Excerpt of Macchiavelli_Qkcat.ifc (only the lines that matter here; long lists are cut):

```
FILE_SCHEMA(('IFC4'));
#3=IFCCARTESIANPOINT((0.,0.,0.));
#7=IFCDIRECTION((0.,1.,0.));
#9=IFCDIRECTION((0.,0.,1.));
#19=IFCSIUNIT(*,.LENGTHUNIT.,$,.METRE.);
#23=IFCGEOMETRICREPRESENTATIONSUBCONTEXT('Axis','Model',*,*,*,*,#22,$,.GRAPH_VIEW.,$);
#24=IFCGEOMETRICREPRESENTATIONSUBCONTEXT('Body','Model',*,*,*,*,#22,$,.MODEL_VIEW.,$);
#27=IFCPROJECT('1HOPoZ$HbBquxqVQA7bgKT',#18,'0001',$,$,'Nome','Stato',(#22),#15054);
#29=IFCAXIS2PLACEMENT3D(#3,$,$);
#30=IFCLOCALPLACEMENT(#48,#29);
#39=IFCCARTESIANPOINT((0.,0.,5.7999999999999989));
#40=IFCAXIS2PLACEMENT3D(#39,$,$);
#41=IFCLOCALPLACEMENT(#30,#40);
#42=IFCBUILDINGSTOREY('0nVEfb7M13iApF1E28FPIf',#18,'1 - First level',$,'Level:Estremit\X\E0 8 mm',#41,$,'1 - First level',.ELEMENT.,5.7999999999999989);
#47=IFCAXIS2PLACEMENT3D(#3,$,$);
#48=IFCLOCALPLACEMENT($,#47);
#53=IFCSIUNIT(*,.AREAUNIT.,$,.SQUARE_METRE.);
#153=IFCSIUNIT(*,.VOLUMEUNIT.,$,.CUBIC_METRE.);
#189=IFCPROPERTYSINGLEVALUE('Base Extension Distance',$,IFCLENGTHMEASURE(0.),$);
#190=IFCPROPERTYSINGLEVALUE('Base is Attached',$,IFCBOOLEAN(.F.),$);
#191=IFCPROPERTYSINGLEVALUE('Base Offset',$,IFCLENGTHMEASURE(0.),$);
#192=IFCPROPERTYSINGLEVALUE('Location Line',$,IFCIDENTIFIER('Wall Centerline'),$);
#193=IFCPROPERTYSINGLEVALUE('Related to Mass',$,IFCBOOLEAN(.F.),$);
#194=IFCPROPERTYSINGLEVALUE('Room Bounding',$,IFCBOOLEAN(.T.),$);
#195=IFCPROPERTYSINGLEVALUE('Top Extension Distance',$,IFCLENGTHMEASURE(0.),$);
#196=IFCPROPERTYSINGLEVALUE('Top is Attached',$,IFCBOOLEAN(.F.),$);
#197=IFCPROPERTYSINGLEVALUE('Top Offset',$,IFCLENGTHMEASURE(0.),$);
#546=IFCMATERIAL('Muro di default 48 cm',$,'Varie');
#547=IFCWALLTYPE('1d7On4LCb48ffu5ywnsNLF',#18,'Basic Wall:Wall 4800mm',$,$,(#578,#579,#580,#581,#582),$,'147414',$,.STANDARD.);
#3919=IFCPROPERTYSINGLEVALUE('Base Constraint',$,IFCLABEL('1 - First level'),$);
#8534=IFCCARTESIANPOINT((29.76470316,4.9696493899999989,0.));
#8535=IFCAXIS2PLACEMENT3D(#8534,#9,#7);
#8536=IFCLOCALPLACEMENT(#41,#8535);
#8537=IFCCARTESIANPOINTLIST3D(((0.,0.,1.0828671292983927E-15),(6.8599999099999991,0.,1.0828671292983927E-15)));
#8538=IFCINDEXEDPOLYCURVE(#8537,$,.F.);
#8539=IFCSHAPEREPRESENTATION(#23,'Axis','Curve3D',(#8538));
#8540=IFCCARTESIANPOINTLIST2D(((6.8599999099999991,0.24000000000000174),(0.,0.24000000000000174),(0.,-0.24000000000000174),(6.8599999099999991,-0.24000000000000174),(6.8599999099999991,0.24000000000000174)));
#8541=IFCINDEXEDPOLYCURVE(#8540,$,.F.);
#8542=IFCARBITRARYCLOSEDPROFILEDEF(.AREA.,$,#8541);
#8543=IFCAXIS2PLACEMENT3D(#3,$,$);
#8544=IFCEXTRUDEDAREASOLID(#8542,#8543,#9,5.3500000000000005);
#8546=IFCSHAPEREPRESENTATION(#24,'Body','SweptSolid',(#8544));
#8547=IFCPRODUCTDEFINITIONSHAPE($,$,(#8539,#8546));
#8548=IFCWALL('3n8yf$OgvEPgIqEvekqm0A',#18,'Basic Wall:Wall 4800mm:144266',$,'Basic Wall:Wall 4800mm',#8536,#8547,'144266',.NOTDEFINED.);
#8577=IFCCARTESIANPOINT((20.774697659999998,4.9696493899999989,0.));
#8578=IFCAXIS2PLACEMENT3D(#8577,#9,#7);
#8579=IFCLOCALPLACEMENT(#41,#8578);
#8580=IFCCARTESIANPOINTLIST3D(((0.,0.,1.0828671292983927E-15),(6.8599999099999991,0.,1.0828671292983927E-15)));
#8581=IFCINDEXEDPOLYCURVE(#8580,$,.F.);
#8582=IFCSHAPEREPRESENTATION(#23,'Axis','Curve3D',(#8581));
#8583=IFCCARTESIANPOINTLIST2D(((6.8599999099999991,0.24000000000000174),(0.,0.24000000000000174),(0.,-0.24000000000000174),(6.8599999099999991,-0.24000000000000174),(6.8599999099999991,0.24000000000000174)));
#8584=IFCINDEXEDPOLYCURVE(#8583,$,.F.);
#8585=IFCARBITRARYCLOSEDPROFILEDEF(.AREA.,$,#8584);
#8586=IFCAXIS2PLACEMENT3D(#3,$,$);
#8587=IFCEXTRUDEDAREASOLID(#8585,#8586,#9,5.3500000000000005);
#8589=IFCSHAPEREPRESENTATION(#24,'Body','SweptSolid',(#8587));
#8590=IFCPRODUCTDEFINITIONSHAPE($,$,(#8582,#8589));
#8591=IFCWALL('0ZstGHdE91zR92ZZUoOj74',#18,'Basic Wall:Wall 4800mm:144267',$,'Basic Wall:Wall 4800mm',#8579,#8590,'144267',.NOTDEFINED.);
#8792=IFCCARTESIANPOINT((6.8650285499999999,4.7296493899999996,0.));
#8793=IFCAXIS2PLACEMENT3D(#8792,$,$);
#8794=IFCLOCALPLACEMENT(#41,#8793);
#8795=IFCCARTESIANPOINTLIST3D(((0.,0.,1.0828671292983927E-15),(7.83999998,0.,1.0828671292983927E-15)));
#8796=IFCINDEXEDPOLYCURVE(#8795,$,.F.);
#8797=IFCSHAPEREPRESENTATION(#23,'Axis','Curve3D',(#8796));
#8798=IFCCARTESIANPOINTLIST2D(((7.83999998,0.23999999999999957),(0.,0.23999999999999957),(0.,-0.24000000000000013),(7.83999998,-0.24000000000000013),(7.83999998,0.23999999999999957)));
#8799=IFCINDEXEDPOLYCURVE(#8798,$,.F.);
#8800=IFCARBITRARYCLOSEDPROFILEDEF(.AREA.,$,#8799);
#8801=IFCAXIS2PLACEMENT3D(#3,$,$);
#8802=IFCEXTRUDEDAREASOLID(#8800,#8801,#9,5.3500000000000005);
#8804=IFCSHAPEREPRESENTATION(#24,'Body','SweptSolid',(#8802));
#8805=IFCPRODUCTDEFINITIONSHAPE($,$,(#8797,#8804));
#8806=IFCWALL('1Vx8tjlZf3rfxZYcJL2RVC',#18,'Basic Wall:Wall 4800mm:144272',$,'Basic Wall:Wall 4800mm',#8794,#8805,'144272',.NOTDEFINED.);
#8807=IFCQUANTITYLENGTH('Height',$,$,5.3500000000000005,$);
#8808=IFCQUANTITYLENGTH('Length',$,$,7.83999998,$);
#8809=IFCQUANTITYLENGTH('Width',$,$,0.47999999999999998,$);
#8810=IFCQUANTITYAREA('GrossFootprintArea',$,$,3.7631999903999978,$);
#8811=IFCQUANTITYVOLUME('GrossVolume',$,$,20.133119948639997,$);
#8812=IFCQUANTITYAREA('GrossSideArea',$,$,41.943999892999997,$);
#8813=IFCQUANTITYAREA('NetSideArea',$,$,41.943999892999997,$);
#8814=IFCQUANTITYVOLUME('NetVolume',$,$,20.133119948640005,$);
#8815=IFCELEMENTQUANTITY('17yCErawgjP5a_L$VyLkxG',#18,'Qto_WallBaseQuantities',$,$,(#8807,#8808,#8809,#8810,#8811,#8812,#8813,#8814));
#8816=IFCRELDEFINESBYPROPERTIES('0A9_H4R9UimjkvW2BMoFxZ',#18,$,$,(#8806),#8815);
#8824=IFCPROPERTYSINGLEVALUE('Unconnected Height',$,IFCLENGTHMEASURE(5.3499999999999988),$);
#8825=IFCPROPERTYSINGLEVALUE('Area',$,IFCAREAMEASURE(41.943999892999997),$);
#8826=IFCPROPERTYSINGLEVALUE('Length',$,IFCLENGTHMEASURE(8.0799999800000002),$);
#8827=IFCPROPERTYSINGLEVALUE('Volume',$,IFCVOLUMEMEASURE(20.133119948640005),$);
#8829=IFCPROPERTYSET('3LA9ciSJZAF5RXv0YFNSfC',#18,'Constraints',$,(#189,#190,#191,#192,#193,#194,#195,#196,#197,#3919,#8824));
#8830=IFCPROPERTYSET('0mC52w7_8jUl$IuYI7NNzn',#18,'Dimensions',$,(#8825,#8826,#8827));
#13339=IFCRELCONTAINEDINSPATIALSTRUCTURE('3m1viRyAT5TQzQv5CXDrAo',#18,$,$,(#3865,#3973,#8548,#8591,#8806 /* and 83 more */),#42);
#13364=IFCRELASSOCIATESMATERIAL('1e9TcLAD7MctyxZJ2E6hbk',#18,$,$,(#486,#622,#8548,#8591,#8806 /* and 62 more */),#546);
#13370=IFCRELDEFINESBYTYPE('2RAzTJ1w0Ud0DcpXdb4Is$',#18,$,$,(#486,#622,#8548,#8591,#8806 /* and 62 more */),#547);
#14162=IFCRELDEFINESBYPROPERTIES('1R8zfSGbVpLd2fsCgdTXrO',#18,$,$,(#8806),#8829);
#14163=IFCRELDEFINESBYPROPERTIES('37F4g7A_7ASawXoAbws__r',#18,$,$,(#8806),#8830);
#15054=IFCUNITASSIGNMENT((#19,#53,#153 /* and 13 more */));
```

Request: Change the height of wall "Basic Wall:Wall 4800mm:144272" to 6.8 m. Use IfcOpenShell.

```python
import ifcopenshell
import ifcopenshell.api.pset
import ifcopenshell.geom
import ifcopenshell.util.element
import ifcopenshell.util.representation
import ifcopenshell.util.shape
import ifcopenshell.util.unit

model = ifcopenshell.open("Macchiavelli_Qkcat.ifc")
unit_scale = ifcopenshell.util.unit.calculate_unit_scale(model)
area_scale = ifcopenshell.util.unit.calculate_unit_scale(model, "AREAUNIT")
volume_scale = ifcopenshell.util.unit.calculate_unit_scale(model, "VOLUMEUNIT")
settings = ifcopenshell.geom.settings()


def volume(element):
    """Net volume in cubic metres, openings subtracted."""
    shape = ifcopenshell.geom.create_shape(settings, element)
    return ifcopenshell.util.shape.get_volume(shape.geometry)


wall = model.by_id(8806)
before = volume(wall)

body = ifcopenshell.util.representation.get_representation(wall, "Model", "Body")
solid = body.Items[0]
old_height = solid.Depth
solid.Depth = 6.8 / unit_scale
after = volume(wall)
thickness = 0.48  # wall thickness in metres

# Update the stored height, areas and volumes.
qto = model.by_id(ifcopenshell.util.element.get_pset(wall, "Qto_WallBaseQuantities", should_inherit=False)["id"])
ifcopenshell.api.pset.edit_qto(model, qto=qto, properties={
    "Height": solid.Depth,
    "GrossVolume": ifcopenshell.util.element.get_pset(wall, "Qto_WallBaseQuantities", "GrossVolume") * solid.Depth / old_height,
    "GrossSideArea": ifcopenshell.util.element.get_pset(wall, "Qto_WallBaseQuantities", "GrossSideArea") * solid.Depth / old_height,
    "NetSideArea": after / thickness / area_scale,
    "NetVolume": after / volume_scale,
})
pset = model.by_id(ifcopenshell.util.element.get_pset(wall, "Constraints", should_inherit=False)["id"])
ifcopenshell.api.pset.edit_pset(model, pset=pset, properties={
    "Unconnected Height": model.create_entity("IfcLengthMeasure", solid.Depth),
})
pset = model.by_id(ifcopenshell.util.element.get_pset(wall, "Dimensions", should_inherit=False)["id"])
ifcopenshell.api.pset.edit_pset(model, pset=pset, properties={
    "Area": model.create_entity("IfcAreaMeasure", after / thickness / area_scale),
    "Volume": model.create_entity("IfcVolumeMeasure", after / volume_scale),
})

print(f"height {old_height:g} -> {solid.Depth:g}, volume {before:.3f} -> {after:.3f} m3")

model.write("Macchiavelli_Qkcat-out.ifc")
```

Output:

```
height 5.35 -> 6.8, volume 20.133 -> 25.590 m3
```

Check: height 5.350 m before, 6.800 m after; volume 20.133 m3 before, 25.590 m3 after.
